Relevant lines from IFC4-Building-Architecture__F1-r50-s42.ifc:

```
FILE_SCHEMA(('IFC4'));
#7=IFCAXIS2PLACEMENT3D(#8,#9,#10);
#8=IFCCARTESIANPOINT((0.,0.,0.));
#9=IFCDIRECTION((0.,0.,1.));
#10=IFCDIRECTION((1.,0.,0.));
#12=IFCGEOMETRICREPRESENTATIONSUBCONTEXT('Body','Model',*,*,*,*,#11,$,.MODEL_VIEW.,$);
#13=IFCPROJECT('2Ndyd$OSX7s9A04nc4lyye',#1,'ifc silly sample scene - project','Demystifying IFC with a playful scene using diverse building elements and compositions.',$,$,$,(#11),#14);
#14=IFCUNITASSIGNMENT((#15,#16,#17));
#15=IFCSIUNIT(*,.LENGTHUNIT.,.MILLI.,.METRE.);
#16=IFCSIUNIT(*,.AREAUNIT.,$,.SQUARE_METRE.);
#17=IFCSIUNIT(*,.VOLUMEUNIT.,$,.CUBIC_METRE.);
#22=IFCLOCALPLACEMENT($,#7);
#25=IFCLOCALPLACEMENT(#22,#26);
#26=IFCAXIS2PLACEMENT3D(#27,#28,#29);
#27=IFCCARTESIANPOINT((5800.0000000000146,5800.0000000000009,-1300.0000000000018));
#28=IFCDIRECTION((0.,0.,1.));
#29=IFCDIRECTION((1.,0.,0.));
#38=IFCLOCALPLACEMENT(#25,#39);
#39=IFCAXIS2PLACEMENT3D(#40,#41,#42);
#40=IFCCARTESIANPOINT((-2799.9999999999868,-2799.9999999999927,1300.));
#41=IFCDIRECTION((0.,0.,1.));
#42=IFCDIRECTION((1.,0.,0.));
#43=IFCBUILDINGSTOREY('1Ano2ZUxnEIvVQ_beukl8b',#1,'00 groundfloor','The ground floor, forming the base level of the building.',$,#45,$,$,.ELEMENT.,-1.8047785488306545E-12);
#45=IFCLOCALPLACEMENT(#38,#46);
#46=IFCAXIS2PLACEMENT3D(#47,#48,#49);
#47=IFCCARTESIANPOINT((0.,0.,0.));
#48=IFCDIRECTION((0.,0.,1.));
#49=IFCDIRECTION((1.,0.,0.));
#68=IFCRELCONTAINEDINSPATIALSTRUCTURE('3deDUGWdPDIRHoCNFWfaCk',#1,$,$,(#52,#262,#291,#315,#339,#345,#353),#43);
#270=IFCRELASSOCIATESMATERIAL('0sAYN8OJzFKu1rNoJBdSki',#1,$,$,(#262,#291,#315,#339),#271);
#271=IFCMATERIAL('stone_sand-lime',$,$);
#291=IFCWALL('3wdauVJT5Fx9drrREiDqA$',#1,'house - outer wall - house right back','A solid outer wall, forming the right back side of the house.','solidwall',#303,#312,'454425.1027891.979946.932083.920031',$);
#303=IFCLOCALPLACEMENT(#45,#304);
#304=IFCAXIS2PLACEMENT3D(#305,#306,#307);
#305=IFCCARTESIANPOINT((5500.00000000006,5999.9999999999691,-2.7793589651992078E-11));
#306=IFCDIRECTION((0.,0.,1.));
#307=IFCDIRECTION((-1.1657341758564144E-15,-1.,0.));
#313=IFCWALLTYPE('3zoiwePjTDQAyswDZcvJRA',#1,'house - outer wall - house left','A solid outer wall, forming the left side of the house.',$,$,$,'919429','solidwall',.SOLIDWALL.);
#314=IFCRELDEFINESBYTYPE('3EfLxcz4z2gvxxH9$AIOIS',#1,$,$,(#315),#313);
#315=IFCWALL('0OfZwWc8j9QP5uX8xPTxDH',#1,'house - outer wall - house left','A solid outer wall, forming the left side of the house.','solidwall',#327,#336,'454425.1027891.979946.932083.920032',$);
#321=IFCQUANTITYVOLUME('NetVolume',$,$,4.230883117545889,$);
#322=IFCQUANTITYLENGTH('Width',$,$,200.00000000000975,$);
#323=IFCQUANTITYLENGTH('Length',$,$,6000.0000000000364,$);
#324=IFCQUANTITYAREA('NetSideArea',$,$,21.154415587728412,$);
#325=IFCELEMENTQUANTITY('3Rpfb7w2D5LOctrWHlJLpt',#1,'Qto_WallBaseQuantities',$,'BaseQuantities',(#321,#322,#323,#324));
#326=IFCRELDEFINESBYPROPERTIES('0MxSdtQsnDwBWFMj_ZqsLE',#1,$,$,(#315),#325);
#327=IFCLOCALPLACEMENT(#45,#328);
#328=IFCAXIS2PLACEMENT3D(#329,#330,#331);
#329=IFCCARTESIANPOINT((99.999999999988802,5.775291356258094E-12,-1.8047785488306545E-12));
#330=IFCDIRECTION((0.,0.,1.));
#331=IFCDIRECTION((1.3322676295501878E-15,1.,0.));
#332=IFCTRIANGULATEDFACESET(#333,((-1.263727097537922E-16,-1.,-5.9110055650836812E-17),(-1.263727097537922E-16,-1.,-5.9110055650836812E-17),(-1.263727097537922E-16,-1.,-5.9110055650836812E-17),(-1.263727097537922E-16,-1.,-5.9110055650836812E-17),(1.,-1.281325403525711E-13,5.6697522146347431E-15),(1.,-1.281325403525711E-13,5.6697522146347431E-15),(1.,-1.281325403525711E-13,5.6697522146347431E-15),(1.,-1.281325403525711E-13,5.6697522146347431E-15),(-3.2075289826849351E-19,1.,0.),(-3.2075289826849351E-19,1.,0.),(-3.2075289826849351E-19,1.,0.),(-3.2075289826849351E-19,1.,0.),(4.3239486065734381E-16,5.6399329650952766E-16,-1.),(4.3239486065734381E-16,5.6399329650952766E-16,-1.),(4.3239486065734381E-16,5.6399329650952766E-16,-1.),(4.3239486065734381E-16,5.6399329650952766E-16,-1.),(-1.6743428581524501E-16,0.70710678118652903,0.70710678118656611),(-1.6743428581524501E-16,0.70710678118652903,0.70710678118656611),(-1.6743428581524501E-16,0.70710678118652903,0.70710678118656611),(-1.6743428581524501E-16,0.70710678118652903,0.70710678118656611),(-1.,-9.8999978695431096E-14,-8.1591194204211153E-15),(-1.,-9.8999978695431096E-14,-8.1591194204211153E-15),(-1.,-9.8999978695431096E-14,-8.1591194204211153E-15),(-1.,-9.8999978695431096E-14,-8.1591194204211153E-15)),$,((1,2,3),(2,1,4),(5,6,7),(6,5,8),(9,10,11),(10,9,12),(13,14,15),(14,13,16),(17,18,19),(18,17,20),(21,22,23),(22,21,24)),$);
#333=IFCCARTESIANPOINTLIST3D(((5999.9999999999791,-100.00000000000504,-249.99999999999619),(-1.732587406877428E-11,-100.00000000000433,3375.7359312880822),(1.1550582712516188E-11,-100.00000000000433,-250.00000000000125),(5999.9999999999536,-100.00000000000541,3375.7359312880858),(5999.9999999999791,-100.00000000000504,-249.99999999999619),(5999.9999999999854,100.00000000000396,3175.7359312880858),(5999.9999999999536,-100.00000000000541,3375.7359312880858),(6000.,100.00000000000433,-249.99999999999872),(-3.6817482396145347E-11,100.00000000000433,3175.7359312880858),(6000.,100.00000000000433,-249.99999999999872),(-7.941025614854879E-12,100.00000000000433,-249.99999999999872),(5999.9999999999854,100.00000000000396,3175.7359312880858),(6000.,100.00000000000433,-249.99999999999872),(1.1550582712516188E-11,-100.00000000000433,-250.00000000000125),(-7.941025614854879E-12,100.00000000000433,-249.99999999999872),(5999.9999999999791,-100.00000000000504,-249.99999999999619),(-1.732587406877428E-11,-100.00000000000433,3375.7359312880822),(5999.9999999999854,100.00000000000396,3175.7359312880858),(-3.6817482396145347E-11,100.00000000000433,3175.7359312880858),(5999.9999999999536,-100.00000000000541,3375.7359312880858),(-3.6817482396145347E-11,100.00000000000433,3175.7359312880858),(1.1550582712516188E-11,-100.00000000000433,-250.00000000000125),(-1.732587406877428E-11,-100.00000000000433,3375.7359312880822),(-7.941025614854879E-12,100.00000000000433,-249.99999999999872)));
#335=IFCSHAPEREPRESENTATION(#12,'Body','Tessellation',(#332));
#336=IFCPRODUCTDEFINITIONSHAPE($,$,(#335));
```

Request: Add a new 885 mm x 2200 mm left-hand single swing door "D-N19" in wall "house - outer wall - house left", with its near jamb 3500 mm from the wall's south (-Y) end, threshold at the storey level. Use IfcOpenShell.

```python
import numpy as np
import ifcopenshell
import ifcopenshell.api.feature
import ifcopenshell.api.geometry
import ifcopenshell.api.pset
import ifcopenshell.api.root
import ifcopenshell.api.spatial
import ifcopenshell.geom
import ifcopenshell.util.element
import ifcopenshell.util.placement
import ifcopenshell.util.representation
import ifcopenshell.util.shape
import ifcopenshell.util.unit

model = ifcopenshell.open("IFC4-Building-Architecture__F1-r50-s42.ifc")
unit_scale = ifcopenshell.util.unit.calculate_unit_scale(model)
area_scale = ifcopenshell.util.unit.calculate_unit_scale(model, "AREAUNIT")
volume_scale = ifcopenshell.util.unit.calculate_unit_scale(model, "VOLUMEUNIT")
settings = ifcopenshell.geom.settings()


def volume(element):
    """Net volume in cubic metres, openings subtracted."""
    shape = ifcopenshell.geom.create_shape(settings, element)
    return ifcopenshell.util.shape.get_volume(shape.geometry)


wall = model.by_guid("0OfZwWc8j9QP5uX8xPTxDH")
storey = ifcopenshell.util.element.get_container(wall, ifc_class="IfcBuildingStorey")
context = ifcopenshell.util.representation.get_context(model, "Model", "Body", "MODEL_VIEW")
before = volume(wall)

width, height, from_end, sill = 0.885, 2.2, 3.5, 0.0  # metres

# The wall runs along its own X axis, and the end named is its -X end.
wall_shape = ifcopenshell.geom.create_shape(settings, wall)
x, y, z = ifcopenshell.util.shape.get_vertices(wall_shape.geometry).T
start = x.min() + from_end
face, thickness = float(y.min()), float(y.max() - y.min())
wall_matrix = ifcopenshell.util.placement.get_local_placement(wall.ObjectPlacement)
level = ifcopenshell.util.placement.get_local_placement(storey.ObjectPlacement)[2, 3]


def in_wall(x, y):
    """Placement at x, y metres in the wall's axes, at sill height."""
    matrix = wall_matrix.copy()
    matrix[:, 3] = wall_matrix @ np.array([x / unit_scale, y / unit_scale, 0.0, 1.0])
    matrix[2, 3] = level + sill / unit_scale
    return matrix


# Opening: a box that overshoots both wall faces by 50 mm.
opening = ifcopenshell.api.root.create_entity(model, ifc_class="IfcOpeningElement", predefined_type="OPENING")
box = ifcopenshell.api.geometry.add_wall_representation(
    model, context=context, length=width, height=height, thickness=thickness + 0.1
)
ifcopenshell.api.geometry.assign_representation(model, product=opening, representation=box)
ifcopenshell.api.geometry.edit_object_placement(model, product=opening, matrix=in_wall(start, face - 0.05), is_si=False)
ifcopenshell.api.feature.add_feature(model, feature=opening, element=wall)

door = ifcopenshell.api.root.create_entity(model, ifc_class="IfcDoor", name="D-N19", predefined_type="DOOR")
door.OverallWidth, door.OverallHeight = width / unit_scale, height / unit_scale
door.OperationType = "SINGLE_SWING_LEFT"
body = ifcopenshell.api.geometry.add_door_representation(
    model,
    context=context,
    overall_width=door.OverallWidth,
    overall_height=door.OverallHeight,
    operation_type="SINGLE_SWING_LEFT",
    lining_properties={"LiningDepth": thickness / unit_scale, "ThresholdDepth": thickness / unit_scale},
)
ifcopenshell.api.geometry.assign_representation(model, product=door, representation=body)
ifcopenshell.api.spatial.assign_container(model, products=[door], relating_structure=storey)
ifcopenshell.api.feature.add_filling(model, opening=opening, element=door)

# The lining spans the wall, so the door starts at the wall face.
ifcopenshell.api.geometry.edit_object_placement(model, product=door, matrix=in_wall(start, face), is_si=False)

after = volume(wall)

# Update the wall's stored quantities.
qto = model.by_id(ifcopenshell.util.element.get_pset(wall, "Qto_WallBaseQuantities", should_inherit=False)["id"])
ifcopenshell.api.pset.edit_qto(model, qto=qto, properties={
    "NetVolume": after / volume_scale,
    "NetSideArea": after / thickness / area_scale,
})

print(f"wall volume {before:.3f} -> {after:.3f} m3")

model.write("IFC4-Building-Architecture__F1-r50-s42_rev.ifc")
```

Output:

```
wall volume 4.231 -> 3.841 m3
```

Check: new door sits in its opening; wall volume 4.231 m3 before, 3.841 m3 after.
